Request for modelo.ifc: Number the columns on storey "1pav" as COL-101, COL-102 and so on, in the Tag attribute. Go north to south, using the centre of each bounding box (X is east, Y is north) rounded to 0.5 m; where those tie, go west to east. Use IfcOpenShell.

First a look at what the model holds.

```python
import ifcopenshell
import ifcopenshell.util.element
import ifcopenshell.util.placement

model = ifcopenshell.open("modelo.ifc")
print(model.schema)
storey = next(s for s in model.by_type("IfcBuildingStorey") if s.Name == "1pav")
columns = [e for e in ifcopenshell.util.element.get_decomposition(storey) if e.is_a("IfcColumn")]
for e in sorted(columns, key=lambda e: e.id()):
    origin = ifcopenshell.util.placement.get_local_placement(e.ObjectPlacement)[:3, 3]
    print(e.id(), e.Tag, e.Name, origin.round(2) + 0.0, sep=" | ")
```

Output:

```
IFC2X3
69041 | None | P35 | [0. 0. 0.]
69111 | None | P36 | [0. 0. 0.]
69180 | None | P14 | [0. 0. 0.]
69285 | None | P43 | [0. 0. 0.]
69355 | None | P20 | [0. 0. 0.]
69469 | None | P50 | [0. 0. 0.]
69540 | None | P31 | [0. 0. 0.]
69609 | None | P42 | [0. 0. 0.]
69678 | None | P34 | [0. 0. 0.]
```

```python
import ifcopenshell
import ifcopenshell.geom
import ifcopenshell.util.element
import ifcopenshell.util.shape

model = ifcopenshell.open("modelo.ifc")
settings = ifcopenshell.geom.settings()
settings.set("use-world-coords", True)


def centre(element):
    shape = ifcopenshell.geom.create_shape(settings, element)
    return ifcopenshell.util.shape.get_bbox_centroid(shape.geometry)


storey = next(s for s in model.by_type("IfcBuildingStorey") if s.Name == "1pav")
columns = [e for e in ifcopenshell.util.element.get_decomposition(storey) if e.is_a("IfcColumn")]

# Insertion points can sit at a corner or the storey origin, so sort by the geometry (in metres).
centres = {e: centre(e) for e in columns}
columns.sort(key=lambda e: (-round(centres[e][1] / 0.5), centres[e][0]))

for i, e in enumerate(columns, start=1):
    number = f"COL-1{i:02d}"
    e.Tag = number
    print(e.id(), number)

model.write("modelo_updated.ifc")
```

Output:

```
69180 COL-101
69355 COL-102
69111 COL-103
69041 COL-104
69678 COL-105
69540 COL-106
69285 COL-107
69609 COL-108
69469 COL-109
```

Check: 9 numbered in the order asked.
